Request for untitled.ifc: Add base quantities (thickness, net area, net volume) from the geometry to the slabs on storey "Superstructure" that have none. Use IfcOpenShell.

First a look at what the model holds.

```python
import ifcopenshell
import ifcopenshell.util.element
import ifcopenshell.util.unit

model = ifcopenshell.open("untitled.ifc")
print(model.schema)
for unit_type in ("LENGTHUNIT", "AREAUNIT", "VOLUMEUNIT"):
    print(unit_type, ifcopenshell.util.unit.calculate_unit_scale(model, unit_type))
storey = next(s for s in model.by_type("IfcBuildingStorey") if s.Name == "Superstructure")
slabs = [e for e in ifcopenshell.util.element.get_decomposition(storey) if e.is_a("IfcSlab")]
for e in sorted(slabs, key=lambda e: e.id()):
    print(e.id(), e.is_a(), e.Name, list(ifcopenshell.util.element.get_psets(e, qtos_only=True)), sep=" | ")
```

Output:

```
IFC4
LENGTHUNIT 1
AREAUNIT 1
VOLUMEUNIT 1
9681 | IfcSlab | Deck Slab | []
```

```python
import ifcopenshell
import ifcopenshell.api.pset
import ifcopenshell.geom
import ifcopenshell.util.element
import ifcopenshell.util.shape
import ifcopenshell.util.unit

model = ifcopenshell.open("untitled.ifc")
unit_scale = ifcopenshell.util.unit.calculate_unit_scale(model)
area_scale = ifcopenshell.util.unit.calculate_unit_scale(model, "AREAUNIT")
volume_scale = ifcopenshell.util.unit.calculate_unit_scale(model, "VOLUMEUNIT")
settings = ifcopenshell.geom.settings()

storey = next(s for s in model.by_type("IfcBuildingStorey") if s.Name == "Superstructure")
slabs = [e for e in ifcopenshell.util.element.get_decomposition(storey) if e.is_a("IfcSlab")]

for e in sorted(slabs, key=lambda e: e.id()):
    if ifcopenshell.util.element.get_psets(e, qtos_only=True, should_inherit=False):
        continue
    # Geometry comes back in metres, in the element's own axes.
    shape = ifcopenshell.geom.create_shape(settings, e)
    values = {
        "Width": ifcopenshell.util.shape.get_z(shape.geometry) / unit_scale,
        "NetArea": ifcopenshell.util.shape.get_footprint_area(shape.geometry) / area_scale,
        "NetVolume": ifcopenshell.util.shape.get_volume(shape.geometry) / volume_scale,
    }
    qto = ifcopenshell.api.pset.add_qto(model, product=e, name="Qto_SlabBaseQuantities")
    ifcopenshell.api.pset.edit_qto(model, qto=qto, properties=values)
    print(e.id(), {k: round(v, 3) for k, v in values.items()})

model.write("untitled-out.ifc")
```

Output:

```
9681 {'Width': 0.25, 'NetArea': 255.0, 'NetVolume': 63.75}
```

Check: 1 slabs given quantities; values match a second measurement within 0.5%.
